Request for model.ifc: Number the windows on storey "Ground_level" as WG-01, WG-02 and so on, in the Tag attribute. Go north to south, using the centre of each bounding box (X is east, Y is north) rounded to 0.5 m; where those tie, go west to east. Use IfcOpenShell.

First a look at what the model holds.

```python
import ifcopenshell
import ifcopenshell.util.element
import ifcopenshell.util.placement

model = ifcopenshell.open("model.ifc")
print(model.schema)
storey = next(s for s in model.by_type("IfcBuildingStorey") if s.Name == "Ground_level")
windows = [e for e in ifcopenshell.util.element.get_decomposition(storey) if e.is_a("IfcWindow")]
for e in sorted(windows, key=lambda e: e.id()):
    origin = ifcopenshell.util.placement.get_local_placement(e.ObjectPlacement)[:3, 3]
    print(e.id(), e.Tag, e.Name, origin.round(2) + 0.0, sep=" | ")
```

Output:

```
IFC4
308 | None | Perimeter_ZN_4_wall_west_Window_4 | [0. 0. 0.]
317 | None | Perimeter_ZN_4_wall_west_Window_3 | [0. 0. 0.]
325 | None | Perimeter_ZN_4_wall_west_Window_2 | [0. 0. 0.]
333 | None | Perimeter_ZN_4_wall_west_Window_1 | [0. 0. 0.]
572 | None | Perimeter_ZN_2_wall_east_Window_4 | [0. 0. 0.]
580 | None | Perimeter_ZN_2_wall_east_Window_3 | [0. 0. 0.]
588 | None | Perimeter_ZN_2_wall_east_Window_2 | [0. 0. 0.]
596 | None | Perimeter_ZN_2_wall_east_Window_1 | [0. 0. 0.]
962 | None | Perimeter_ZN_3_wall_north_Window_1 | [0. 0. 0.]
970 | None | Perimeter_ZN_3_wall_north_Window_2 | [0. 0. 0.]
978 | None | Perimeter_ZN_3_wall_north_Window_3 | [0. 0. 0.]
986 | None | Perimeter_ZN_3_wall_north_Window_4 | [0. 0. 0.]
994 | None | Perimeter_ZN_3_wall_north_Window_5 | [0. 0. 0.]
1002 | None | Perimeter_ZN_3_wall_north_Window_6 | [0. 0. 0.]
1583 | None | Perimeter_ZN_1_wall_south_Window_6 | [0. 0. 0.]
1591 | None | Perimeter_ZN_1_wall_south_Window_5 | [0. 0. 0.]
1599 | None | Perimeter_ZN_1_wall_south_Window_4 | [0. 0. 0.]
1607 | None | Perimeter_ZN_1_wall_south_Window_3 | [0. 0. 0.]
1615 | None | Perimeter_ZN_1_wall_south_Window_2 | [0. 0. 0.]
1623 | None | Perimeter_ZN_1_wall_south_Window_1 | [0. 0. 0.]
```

```python
import ifcopenshell
import ifcopenshell.geom
import ifcopenshell.util.element
import ifcopenshell.util.shape

model = ifcopenshell.open("model.ifc")
settings = ifcopenshell.geom.settings()
settings.set("use-world-coords", True)


def centre(element):
    shape = ifcopenshell.geom.create_shape(settings, element)
    return ifcopenshell.util.shape.get_bbox_centroid(shape.geometry)


storey = next(s for s in model.by_type("IfcBuildingStorey") if s.Name == "Ground_level")
windows = [e for e in ifcopenshell.util.element.get_decomposition(storey) if e.is_a("IfcWindow")]

# Insertion points can sit at a corner or the storey origin, so sort by the geometry (in metres).
centres = {e: centre(e) for e in windows}
windows.sort(key=lambda e: (-round(centres[e][1] / 0.5), centres[e][0]))

for i, e in enumerate(windows, start=1):
    number = f"WG-{i:02d}"
    e.Tag = number
    print(e.id(), number)

model.write("model_updated.ifc")
```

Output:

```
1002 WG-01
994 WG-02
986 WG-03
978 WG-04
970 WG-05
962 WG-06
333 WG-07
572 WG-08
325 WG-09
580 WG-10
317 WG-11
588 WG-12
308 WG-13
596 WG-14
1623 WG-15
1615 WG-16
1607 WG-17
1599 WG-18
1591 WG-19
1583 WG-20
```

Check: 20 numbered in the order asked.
